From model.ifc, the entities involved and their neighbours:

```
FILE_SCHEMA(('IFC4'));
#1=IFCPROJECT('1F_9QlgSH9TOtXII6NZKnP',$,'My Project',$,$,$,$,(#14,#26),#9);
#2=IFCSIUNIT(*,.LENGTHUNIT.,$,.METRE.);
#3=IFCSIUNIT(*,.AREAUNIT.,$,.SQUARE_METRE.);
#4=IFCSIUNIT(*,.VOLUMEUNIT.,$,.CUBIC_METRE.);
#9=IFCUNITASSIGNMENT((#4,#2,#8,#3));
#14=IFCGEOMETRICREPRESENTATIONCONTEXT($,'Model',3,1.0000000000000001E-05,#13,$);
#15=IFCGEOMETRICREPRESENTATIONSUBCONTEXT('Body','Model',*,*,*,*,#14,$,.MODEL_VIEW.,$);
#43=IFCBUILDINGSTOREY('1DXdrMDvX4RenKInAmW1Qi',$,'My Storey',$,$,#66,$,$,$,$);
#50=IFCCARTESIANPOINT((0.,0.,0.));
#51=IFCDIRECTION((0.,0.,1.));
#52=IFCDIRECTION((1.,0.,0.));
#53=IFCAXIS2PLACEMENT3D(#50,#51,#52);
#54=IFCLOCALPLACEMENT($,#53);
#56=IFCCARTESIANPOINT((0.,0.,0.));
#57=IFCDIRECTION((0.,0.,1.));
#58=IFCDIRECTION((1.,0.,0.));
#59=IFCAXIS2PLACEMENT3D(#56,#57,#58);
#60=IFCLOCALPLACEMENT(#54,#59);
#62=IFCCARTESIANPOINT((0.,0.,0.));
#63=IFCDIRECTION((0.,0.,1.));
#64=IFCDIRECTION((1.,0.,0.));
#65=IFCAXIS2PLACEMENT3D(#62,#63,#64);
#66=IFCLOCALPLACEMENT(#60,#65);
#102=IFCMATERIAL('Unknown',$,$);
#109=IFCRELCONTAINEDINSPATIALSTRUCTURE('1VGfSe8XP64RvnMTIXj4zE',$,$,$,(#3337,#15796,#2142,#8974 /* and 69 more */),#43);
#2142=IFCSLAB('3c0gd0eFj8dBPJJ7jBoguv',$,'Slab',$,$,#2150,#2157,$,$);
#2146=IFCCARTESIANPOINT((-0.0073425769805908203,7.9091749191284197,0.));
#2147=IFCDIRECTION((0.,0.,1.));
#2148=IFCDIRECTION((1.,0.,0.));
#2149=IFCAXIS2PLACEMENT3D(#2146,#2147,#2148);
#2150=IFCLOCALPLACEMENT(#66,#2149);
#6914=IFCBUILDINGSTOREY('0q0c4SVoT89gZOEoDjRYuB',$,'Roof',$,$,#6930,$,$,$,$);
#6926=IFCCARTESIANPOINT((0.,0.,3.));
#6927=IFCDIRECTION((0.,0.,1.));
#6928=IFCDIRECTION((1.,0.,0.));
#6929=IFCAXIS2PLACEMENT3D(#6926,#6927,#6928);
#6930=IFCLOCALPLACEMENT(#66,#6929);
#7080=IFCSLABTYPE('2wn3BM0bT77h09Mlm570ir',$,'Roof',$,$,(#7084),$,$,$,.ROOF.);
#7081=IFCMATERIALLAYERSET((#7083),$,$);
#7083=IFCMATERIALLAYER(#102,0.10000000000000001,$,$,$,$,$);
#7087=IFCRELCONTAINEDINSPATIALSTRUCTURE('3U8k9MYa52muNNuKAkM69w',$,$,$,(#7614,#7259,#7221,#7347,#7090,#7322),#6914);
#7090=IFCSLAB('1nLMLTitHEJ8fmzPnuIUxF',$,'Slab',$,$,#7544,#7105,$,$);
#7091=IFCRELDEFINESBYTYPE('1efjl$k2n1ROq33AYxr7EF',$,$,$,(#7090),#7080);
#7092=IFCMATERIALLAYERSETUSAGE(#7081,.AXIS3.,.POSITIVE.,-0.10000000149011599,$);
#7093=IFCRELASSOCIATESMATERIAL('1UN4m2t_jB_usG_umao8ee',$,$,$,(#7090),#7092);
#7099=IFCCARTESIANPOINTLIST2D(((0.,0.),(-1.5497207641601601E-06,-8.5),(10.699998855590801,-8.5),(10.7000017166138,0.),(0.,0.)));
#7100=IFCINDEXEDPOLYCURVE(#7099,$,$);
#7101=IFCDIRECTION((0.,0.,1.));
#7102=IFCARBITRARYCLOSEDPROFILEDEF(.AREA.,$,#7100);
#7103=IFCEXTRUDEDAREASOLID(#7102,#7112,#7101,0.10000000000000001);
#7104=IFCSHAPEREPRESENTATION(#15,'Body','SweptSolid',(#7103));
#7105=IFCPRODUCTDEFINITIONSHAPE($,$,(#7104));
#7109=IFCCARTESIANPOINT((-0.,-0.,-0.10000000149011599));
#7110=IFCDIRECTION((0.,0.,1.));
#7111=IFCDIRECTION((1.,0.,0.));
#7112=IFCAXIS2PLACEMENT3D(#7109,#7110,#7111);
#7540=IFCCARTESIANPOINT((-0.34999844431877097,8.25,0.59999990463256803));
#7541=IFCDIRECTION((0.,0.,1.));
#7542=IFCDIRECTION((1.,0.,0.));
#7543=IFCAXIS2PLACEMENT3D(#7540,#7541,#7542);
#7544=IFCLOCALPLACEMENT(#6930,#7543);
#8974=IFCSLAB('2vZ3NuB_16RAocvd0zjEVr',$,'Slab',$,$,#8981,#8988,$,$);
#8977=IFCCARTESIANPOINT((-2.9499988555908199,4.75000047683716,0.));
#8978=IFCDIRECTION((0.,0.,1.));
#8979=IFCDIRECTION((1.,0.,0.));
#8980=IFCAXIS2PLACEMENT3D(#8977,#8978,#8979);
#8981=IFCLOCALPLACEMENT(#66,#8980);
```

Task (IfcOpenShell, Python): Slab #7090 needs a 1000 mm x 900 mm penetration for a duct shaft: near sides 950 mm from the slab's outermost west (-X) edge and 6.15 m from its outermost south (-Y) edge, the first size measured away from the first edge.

```python
import numpy as np
import ifcopenshell
import ifcopenshell.api.feature
import ifcopenshell.api.geometry
import ifcopenshell.api.root
import ifcopenshell.geom
import ifcopenshell.util.placement
import ifcopenshell.util.representation
import ifcopenshell.util.shape
import ifcopenshell.util.unit

model = ifcopenshell.open("model.ifc")
unit_scale = ifcopenshell.util.unit.calculate_unit_scale(model)
settings = ifcopenshell.geom.settings()


def volume(element):
    """Net volume in cubic metres, openings subtracted."""
    shape = ifcopenshell.geom.create_shape(settings, element)
    return ifcopenshell.util.shape.get_volume(shape.geometry)


slab = model.by_guid("1nLMLTitHEJ8fmzPnuIUxF")
before = volume(slab)

# Extent in the slab's own axes, in metres. The edges named are its -X and -Y sides.
slab_shape = ifcopenshell.geom.create_shape(settings, slab)
vertices = ifcopenshell.util.shape.get_vertices(slab_shape.geometry)
x_min, y_min, bottom = vertices.min(axis=0)
top = vertices[:, 2].max()

opening = ifcopenshell.api.root.create_entity(model, ifc_class="IfcOpeningElement", name="Duct shaft opening", predefined_type="OPENING")
context = ifcopenshell.util.representation.get_context(model, "Model", "Body", "MODEL_VIEW")
width, depth = 1, 0.9
outline = [(0.0, 0.0), (width, 0.0), (width, depth), (0.0, depth), (0.0, 0.0)]
# Overshoot both faces by 50 mm so the cut is clean.
shape = ifcopenshell.api.geometry.add_slab_representation(
    model, context=context, depth=top - bottom + 0.1, polyline=outline
)
ifcopenshell.api.geometry.assign_representation(model, product=opening, representation=shape)

matrix = ifcopenshell.util.placement.get_local_placement(slab.ObjectPlacement)
matrix[:, 3] = matrix @ np.append(np.array([x_min + 0.95, y_min + 6.15, bottom - 0.05]) / unit_scale, 1.0)
ifcopenshell.api.geometry.edit_object_placement(model, product=opening, matrix=matrix, is_si=False)
ifcopenshell.api.feature.add_feature(model, feature=opening, element=slab)

after = volume(slab)

print(f"slab volume {before:.3f} -> {after:.3f} m3")

model.write("model-out.ifc")
```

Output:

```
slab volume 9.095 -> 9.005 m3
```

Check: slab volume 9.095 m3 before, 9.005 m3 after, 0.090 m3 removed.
